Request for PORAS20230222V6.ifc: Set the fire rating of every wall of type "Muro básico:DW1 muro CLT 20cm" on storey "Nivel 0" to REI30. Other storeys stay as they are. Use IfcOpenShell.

First a look at what the model holds.

```python
import ifcopenshell
import ifcopenshell.util.element

model = ifcopenshell.open("PORAS20230222V6.ifc")
print(model.schema)
storey = next(s for s in model.by_type("IfcBuildingStorey") if s.Name == "Nivel 0")
walls = [e for e in ifcopenshell.util.element.get_decomposition(storey) if e.is_a("IfcWall")]
seen = {}
for e in walls:
    element_type = ifcopenshell.util.element.get_type(e)
    key = (element_type.Name if element_type != e and element_type else None, ifcopenshell.util.element.get_pset(e, "Pset_WallCommon", "FireRating"))
    seen[key] = seen.get(key, 0) + 1
for (name, value), count in sorted(seen.items(), key=str):
    print(count, "x", name, "|", value)
```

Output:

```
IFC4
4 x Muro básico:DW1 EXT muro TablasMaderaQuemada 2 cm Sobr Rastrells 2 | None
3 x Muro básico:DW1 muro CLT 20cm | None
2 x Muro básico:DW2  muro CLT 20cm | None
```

```python
import ifcopenshell
import ifcopenshell.api.pset
import ifcopenshell.util.element

model = ifcopenshell.open("PORAS20230222V6.ifc")

storey = next(s for s in model.by_type("IfcBuildingStorey") if s.Name == "Nivel 0")
walls = [e for e in ifcopenshell.util.element.get_decomposition(storey) if e.is_a("IfcWall")]

count = 0
for e in walls:
    element_type = ifcopenshell.util.element.get_type(e)
    if element_type in (None, e) or element_type.Name != "Muro básico:DW1 muro CLT 20cm":
        continue
    # add_pset returns the element's existing set when there is one.
    pset = ifcopenshell.api.pset.add_pset(model, product=e, name="Pset_WallCommon")
    ifcopenshell.api.pset.edit_pset(model, pset=pset, properties={"FireRating": "REI30"})
    count += 1

print(count, "walls updated")

model.write("PORAS20230222V6_edited.ifc")
```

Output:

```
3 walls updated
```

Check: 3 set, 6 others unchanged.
